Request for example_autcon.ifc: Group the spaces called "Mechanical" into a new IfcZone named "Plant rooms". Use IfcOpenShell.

First a look at what the model holds.

```python
import ifcopenshell

model = ifcopenshell.open("example_autcon.ifc")
print(model.schema)
seen = {}
for space in model.by_type("IfcSpace"):
    seen[space.LongName] = seen.get(space.LongName, 0) + 1
for name, count in sorted(seen.items(), key=str):
    print(count, "x", name)
print("zones:", [z.Name for z in model.by_type("IfcZone")][:20])
```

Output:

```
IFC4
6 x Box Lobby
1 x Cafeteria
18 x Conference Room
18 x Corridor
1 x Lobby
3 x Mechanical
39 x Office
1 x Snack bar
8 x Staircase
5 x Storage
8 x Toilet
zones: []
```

```python
import ifcopenshell
import ifcopenshell.api.group
import ifcopenshell.api.root

model = ifcopenshell.open("example_autcon.ifc")

names = {"Mechanical"}
spaces = [s for s in model.by_type("IfcSpace") if s.LongName in names]

zone = ifcopenshell.api.root.create_entity(model, ifc_class="IfcZone", name="Plant rooms")
ifcopenshell.api.group.assign_group(model, products=spaces, group=zone)
print(len(spaces), "spaces in", zone.Name)

model.write("example_autcon-out.ifc")
```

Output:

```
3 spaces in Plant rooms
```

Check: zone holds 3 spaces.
